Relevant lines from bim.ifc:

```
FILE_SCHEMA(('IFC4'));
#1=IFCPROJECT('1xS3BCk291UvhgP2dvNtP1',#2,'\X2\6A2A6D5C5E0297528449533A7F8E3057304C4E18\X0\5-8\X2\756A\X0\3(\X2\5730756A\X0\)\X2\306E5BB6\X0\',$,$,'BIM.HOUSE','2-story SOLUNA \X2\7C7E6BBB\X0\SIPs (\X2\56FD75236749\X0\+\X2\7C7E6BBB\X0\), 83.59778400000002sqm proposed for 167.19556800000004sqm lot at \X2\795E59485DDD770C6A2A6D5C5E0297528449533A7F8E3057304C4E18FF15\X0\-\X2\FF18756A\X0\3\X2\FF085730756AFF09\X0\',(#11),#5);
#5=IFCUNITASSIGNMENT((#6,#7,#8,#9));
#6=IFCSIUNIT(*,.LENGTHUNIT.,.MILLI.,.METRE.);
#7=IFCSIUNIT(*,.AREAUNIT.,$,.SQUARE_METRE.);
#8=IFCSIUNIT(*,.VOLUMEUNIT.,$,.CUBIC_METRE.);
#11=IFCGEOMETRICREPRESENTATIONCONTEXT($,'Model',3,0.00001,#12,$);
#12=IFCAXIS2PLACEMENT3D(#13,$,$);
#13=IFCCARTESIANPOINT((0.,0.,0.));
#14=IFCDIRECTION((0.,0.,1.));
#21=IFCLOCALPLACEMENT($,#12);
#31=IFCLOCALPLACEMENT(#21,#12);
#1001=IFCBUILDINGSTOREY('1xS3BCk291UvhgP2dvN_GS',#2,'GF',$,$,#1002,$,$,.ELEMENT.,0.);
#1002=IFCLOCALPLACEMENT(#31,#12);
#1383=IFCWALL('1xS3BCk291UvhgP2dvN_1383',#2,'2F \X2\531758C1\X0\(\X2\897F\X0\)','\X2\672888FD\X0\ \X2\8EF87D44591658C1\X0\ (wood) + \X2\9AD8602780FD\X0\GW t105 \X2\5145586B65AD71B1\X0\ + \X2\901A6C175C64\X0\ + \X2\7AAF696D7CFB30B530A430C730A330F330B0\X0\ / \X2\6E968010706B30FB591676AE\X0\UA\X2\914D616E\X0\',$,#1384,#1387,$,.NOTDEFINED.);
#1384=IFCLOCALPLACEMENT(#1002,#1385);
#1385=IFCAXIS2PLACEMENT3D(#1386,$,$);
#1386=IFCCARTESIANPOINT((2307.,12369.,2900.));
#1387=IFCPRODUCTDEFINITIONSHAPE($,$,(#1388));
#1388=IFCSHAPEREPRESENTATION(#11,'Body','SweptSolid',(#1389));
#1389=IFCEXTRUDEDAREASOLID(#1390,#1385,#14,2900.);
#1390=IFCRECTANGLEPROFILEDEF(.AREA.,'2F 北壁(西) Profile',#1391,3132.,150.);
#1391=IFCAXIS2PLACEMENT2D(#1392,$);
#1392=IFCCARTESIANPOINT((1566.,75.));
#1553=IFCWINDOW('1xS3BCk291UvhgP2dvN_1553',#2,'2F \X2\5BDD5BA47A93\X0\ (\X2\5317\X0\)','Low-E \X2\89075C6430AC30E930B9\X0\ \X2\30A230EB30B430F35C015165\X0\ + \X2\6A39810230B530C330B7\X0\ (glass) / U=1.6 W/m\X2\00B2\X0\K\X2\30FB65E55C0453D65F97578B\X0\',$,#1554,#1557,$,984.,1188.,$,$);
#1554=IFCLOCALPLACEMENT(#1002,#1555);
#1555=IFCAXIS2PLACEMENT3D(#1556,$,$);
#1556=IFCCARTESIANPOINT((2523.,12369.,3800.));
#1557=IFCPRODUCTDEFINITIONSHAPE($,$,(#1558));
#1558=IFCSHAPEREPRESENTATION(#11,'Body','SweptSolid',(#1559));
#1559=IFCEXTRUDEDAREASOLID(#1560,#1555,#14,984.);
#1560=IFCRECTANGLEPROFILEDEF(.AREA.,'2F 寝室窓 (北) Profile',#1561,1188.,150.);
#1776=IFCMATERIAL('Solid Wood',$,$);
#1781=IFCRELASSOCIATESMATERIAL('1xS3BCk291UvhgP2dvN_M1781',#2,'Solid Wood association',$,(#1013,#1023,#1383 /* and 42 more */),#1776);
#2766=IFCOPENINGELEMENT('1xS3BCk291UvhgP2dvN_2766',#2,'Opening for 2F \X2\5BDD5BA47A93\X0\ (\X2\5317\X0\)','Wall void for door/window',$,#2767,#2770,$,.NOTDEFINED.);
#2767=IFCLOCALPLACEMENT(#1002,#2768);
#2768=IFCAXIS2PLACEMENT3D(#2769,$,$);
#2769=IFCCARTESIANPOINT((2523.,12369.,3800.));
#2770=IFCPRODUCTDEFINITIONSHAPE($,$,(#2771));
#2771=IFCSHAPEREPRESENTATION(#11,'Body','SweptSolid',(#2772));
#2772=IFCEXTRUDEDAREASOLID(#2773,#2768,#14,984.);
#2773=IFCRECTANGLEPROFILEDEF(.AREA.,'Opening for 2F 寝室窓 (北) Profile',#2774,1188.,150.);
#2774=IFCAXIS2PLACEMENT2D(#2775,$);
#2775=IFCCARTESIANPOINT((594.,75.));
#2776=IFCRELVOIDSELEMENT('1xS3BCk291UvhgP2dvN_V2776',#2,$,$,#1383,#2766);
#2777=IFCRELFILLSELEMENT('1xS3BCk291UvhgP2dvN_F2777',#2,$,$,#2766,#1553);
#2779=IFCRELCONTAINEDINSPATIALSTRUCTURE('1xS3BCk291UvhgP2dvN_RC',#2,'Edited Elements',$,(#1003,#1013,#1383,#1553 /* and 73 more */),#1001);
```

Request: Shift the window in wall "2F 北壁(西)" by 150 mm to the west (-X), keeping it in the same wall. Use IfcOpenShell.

```python
import ifcopenshell
import ifcopenshell.api.geometry
import ifcopenshell.util.placement
import ifcopenshell.util.unit

model = ifcopenshell.open("bim.ifc")
unit_scale = ifcopenshell.util.unit.calculate_unit_scale(model)

window = model.by_id(1553)
opening = window.FillsVoids[0].RelatingOpeningElement
wall = opening.VoidsElements[0].RelatingBuildingElement

wall_matrix = ifcopenshell.util.placement.get_local_placement(wall.ObjectPlacement)
shift = wall_matrix[:3, 0] * -0.15 / unit_scale
before = ifcopenshell.util.placement.get_local_placement(window.ObjectPlacement)[:3, 3].copy()

# The window is not placed relative to its opening, so move both.
for product in (opening, window):
    matrix = ifcopenshell.util.placement.get_local_placement(product.ObjectPlacement)
    matrix[:3, 3] += shift
    ifcopenshell.api.geometry.edit_object_placement(model, product=product, matrix=matrix, is_si=False)

after = ifcopenshell.util.placement.get_local_placement(window.ObjectPlacement)[:3, 3]
print("window moved by", (after - before).round(3) + 0.0)

model.write("bim_v2.ifc")
```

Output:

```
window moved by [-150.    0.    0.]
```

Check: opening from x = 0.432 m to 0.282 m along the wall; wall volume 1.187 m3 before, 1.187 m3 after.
